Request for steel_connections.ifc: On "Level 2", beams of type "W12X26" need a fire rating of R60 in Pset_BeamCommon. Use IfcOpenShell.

First a look at what the model holds.

```python
import ifcopenshell
import ifcopenshell.util.element

model = ifcopenshell.open("steel_connections.ifc")
print(model.schema)
storey = next(s for s in model.by_type("IfcBuildingStorey") if s.Name == "Level 2")
beams = [e for e in ifcopenshell.util.element.get_decomposition(storey) if e.is_a("IfcBeam")]
seen = {}
for e in beams:
    element_type = ifcopenshell.util.element.get_type(e)
    key = (element_type.Name if element_type != e and element_type else None, ifcopenshell.util.element.get_pset(e, "Pset_BeamCommon", "FireRating"))
    seen[key] = seen.get(key, 0) + 1
for (name, value), count in sorted(seen.items(), key=str):
    print(count, "x", name, "|", value)
```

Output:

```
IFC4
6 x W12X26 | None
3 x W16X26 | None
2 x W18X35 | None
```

```python
import ifcopenshell
import ifcopenshell.api.pset
import ifcopenshell.util.element

model = ifcopenshell.open("steel_connections.ifc")

storey = next(s for s in model.by_type("IfcBuildingStorey") if s.Name == "Level 2")
beams = [e for e in ifcopenshell.util.element.get_decomposition(storey) if e.is_a("IfcBeam")]

count = 0
for e in beams:
    element_type = ifcopenshell.util.element.get_type(e)
    if element_type in (None, e) or element_type.Name != "W12X26":
        continue
    # add_pset returns the element's existing set when there is one.
    pset = ifcopenshell.api.pset.add_pset(model, product=e, name="Pset_BeamCommon")
    ifcopenshell.api.pset.edit_pset(model, pset=pset, properties={"FireRating": "R60"})
    count += 1

print(count, "beams updated")

model.write("steel_connections-out.ifc")
```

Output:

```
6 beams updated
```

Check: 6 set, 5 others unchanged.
